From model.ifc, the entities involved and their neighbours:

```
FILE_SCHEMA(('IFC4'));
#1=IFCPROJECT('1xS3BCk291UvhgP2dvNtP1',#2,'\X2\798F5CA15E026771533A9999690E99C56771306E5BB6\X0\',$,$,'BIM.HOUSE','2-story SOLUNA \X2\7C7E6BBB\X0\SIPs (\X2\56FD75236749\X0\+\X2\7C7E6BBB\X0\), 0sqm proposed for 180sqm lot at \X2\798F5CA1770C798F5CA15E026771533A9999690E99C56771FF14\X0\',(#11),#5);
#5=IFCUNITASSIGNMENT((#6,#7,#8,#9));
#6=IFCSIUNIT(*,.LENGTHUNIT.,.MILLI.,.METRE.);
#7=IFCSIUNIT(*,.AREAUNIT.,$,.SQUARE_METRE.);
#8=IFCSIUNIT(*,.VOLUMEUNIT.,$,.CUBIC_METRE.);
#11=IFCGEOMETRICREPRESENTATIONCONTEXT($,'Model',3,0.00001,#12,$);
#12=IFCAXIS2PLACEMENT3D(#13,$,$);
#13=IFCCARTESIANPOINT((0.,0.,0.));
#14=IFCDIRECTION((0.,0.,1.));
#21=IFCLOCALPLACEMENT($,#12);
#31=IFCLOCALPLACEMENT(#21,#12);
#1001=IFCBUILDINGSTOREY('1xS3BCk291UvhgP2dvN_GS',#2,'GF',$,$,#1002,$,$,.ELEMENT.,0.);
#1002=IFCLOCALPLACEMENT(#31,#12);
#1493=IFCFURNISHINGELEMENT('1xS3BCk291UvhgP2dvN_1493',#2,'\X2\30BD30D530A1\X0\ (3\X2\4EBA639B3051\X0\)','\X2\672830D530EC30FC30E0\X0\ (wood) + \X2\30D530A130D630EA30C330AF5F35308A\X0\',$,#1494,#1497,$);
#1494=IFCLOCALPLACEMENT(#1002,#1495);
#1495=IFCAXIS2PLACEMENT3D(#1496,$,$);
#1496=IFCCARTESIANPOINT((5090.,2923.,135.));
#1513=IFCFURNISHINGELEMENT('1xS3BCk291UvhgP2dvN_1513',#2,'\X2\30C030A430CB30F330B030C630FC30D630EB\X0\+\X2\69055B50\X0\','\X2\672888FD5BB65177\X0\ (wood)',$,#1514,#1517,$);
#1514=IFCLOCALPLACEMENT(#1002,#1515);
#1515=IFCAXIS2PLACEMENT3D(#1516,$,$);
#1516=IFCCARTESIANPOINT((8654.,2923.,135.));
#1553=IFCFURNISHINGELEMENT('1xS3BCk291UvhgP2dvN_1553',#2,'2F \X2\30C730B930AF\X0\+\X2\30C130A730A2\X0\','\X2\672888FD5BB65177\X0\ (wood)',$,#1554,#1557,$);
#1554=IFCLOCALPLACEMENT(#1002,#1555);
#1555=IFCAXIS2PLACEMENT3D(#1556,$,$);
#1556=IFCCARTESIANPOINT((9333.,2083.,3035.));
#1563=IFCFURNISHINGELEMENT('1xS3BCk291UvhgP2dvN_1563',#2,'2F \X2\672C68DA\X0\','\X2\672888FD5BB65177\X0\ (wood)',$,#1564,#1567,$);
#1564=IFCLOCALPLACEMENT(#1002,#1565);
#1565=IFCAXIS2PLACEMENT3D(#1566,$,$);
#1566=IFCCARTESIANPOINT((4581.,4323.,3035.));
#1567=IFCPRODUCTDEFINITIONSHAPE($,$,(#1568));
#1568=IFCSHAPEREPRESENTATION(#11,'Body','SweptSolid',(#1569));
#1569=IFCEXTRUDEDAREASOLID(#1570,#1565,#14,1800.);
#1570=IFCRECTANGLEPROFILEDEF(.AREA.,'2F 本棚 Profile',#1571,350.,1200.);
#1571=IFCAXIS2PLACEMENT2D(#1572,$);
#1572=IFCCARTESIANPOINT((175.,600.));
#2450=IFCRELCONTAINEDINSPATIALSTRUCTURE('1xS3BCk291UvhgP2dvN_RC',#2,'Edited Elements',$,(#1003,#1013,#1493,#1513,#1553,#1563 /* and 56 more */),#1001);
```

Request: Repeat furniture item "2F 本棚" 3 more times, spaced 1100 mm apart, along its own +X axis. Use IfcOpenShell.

```python
import ifcopenshell
import ifcopenshell.api.geometry
import ifcopenshell.api.root
import ifcopenshell.util.element
import ifcopenshell.util.placement
import ifcopenshell.util.unit

model = ifcopenshell.open("model.ifc")
unit_scale = ifcopenshell.util.unit.calculate_unit_scale(model)


def reuse_history(source, copy):
    """copy_class also copies each property set's owner history, people and application; keep the originals."""
    for rel in copy.IsDefinedBy:
        if rel.is_a("IfcRelDefinesByProperties") and (history := rel.RelatingPropertyDefinition.OwnerHistory):
            rel.RelatingPropertyDefinition.OwnerHistory = source.OwnerHistory
            ifcopenshell.util.element.remove_deep2(model, history)


source = model.by_guid("1xS3BCk291UvhgP2dvN_1563")
base = ifcopenshell.util.placement.get_local_placement(source.ObjectPlacement)
step = base[:3, 0] * 1.1 / unit_scale

for i in range(1, 4):
    copy = ifcopenshell.api.root.copy_class(model, product=source)
    copy.Representation = ifcopenshell.util.element.copy_deep(
        model, source.Representation, exclude=["IfcGeometricRepresentationContext", "IfcRepresentationMap"]
    )
    reuse_history(source, copy)
    matrix = base.copy()
    matrix[:3, 3] += i * step
    print("added at", matrix[:3, 3].round(3) + 0.0)
    ifcopenshell.api.geometry.edit_object_placement(model, product=copy, matrix=matrix, is_si=False)

model.write("model_rev.ifc")
```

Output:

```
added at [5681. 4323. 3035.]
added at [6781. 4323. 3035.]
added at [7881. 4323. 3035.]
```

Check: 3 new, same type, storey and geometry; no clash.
